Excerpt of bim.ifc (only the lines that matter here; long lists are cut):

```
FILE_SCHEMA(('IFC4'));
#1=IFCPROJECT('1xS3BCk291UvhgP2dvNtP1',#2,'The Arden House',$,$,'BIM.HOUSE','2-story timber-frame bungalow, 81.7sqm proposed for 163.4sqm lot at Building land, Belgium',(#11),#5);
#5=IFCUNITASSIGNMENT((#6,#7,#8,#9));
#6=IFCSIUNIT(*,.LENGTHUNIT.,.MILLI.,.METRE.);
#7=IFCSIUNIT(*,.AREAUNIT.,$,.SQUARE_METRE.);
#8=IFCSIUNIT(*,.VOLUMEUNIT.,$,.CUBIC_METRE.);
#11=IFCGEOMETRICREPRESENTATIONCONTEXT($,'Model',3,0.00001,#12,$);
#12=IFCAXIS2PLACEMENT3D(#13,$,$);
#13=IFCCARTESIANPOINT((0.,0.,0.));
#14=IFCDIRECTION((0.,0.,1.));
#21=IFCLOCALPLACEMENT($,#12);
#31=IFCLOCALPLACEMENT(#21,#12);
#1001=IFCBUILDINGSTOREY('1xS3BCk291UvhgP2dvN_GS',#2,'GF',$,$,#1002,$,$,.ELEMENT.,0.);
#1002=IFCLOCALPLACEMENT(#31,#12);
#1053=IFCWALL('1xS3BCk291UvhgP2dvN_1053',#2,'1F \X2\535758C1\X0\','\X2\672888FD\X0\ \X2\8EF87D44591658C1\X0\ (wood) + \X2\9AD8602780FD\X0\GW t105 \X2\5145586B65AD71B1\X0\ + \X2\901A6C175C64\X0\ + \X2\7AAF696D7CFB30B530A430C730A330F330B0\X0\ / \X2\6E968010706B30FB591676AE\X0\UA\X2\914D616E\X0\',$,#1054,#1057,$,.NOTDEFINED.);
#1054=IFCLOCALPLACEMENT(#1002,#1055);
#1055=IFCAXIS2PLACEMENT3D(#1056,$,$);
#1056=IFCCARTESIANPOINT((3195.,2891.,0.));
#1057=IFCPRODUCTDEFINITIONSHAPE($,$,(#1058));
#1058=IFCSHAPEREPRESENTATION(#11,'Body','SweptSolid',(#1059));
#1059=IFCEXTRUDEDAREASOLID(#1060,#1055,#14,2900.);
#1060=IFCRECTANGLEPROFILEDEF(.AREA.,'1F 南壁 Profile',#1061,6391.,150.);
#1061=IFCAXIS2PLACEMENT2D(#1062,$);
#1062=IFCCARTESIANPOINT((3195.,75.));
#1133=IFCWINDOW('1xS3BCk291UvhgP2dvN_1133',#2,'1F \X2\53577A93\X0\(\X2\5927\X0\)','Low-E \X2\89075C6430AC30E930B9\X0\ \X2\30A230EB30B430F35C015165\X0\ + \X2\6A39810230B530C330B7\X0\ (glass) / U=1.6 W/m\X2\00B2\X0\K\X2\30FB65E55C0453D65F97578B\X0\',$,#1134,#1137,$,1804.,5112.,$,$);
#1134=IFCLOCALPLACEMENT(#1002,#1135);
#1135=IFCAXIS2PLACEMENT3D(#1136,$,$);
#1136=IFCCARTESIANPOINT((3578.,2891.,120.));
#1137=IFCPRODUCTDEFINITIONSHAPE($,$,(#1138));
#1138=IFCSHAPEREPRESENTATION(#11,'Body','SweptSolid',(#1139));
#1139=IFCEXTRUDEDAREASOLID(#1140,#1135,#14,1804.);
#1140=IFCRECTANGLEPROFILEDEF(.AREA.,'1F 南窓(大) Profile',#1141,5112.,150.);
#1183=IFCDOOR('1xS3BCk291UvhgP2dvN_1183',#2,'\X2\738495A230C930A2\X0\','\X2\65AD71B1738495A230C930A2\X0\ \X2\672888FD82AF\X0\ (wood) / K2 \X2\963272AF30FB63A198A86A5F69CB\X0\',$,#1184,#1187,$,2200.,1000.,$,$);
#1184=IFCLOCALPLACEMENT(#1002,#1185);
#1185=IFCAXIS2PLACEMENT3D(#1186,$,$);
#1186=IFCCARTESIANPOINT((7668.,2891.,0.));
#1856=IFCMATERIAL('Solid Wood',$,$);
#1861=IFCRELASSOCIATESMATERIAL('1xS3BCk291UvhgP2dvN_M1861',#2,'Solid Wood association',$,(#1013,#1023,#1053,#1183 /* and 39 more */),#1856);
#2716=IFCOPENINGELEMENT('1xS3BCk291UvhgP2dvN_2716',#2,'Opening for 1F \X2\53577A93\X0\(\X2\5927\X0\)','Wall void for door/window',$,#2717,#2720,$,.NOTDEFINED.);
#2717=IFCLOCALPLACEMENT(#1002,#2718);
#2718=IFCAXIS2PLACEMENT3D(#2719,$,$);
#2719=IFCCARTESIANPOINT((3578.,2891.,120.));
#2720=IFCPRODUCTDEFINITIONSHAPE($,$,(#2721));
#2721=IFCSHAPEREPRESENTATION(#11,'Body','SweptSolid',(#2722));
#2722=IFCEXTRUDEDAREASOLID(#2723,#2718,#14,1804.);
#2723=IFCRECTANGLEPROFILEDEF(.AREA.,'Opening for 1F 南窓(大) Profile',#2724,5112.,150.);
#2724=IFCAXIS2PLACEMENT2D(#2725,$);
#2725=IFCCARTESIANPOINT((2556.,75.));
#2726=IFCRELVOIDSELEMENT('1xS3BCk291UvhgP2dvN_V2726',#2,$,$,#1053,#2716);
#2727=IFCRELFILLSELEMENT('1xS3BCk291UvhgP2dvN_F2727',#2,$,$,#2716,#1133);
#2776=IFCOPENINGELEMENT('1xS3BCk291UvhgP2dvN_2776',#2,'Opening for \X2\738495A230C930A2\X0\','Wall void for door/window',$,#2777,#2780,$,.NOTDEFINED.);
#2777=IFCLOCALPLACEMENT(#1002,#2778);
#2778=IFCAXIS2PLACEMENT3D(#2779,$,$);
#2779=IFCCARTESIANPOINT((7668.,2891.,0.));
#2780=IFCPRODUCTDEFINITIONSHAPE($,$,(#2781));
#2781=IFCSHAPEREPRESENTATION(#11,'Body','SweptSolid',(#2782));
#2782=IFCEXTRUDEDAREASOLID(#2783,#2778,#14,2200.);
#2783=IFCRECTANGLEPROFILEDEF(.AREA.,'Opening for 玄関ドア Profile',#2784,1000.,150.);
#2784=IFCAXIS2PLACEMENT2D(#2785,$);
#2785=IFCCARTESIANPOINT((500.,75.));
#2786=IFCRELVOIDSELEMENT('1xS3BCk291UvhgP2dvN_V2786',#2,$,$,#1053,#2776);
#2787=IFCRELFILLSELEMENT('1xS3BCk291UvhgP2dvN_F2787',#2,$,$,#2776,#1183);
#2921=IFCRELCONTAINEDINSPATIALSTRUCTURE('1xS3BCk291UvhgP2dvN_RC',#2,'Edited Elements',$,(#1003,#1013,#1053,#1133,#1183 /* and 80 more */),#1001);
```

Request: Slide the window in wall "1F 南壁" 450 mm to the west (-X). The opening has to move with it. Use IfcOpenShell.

```python
import ifcopenshell
import ifcopenshell.api.geometry
import ifcopenshell.util.placement

model = ifcopenshell.open("bim.ifc")

window = model.by_id(1133)
opening = window.FillsVoids[0].RelatingOpeningElement
wall = opening.VoidsElements[0].RelatingBuildingElement

wall_matrix = ifcopenshell.util.placement.get_local_placement(wall.ObjectPlacement)
shift = wall_matrix[:3, 0] * -450.0
before = ifcopenshell.util.placement.get_local_placement(window.ObjectPlacement)[:3, 3].copy()

# The window is not placed relative to its opening, so move both.
for product in (opening, window):
    matrix = ifcopenshell.util.placement.get_local_placement(product.ObjectPlacement)
    matrix[:3, 3] += shift
    ifcopenshell.api.geometry.edit_object_placement(model, product=product, matrix=matrix, is_si=False)

after = ifcopenshell.util.placement.get_local_placement(window.ObjectPlacement)[:3, 3]
print("window moved by", (after - before).round(3) + 0.0)

model.write("bim_rev.ifc")
```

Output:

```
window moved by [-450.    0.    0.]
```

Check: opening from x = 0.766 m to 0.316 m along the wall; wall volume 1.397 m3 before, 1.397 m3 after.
